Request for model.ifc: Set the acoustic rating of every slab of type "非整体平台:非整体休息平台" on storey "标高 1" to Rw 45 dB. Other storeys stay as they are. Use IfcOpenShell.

First a look at what the model holds.

```python
import ifcopenshell
import ifcopenshell.util.element

model = ifcopenshell.open("model.ifc")
print(model.schema)
storey = next(s for s in model.by_type("IfcBuildingStorey") if s.Name == "标高 1")
slabs = [e for e in ifcopenshell.util.element.get_decomposition(storey) if e.is_a("IfcSlab")]
seen = {}
for e in slabs:
    element_type = ifcopenshell.util.element.get_type(e)
    key = (element_type.Name if element_type != e and element_type else None, ifcopenshell.util.element.get_pset(e, "Pset_SlabCommon", "AcousticRating"))
    seen[key] = seen.get(key, 0) + 1
for (name, value), count in sorted(seen.items(), key=str):
    print(count, "x", name, "|", value)
```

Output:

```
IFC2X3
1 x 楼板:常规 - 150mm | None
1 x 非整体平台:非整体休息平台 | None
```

```python
import ifcopenshell
import ifcopenshell.api.pset
import ifcopenshell.util.element

model = ifcopenshell.open("model.ifc")

storey = next(s for s in model.by_type("IfcBuildingStorey") if s.Name == "标高 1")
slabs = [e for e in ifcopenshell.util.element.get_decomposition(storey) if e.is_a("IfcSlab")]

count = 0
for e in slabs:
    element_type = ifcopenshell.util.element.get_type(e)
    if element_type in (None, e) or element_type.Name != "非整体平台:非整体休息平台":
        continue
    # add_pset returns the element's existing set when there is one.
    pset = ifcopenshell.api.pset.add_pset(model, product=e, name="Pset_SlabCommon")
    ifcopenshell.api.pset.edit_pset(model, pset=pset, properties={"AcousticRating": "Rw 45 dB"})
    count += 1

print(count, "slabs updated")

model.write("model_rev.ifc")
```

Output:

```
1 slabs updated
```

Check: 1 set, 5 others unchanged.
